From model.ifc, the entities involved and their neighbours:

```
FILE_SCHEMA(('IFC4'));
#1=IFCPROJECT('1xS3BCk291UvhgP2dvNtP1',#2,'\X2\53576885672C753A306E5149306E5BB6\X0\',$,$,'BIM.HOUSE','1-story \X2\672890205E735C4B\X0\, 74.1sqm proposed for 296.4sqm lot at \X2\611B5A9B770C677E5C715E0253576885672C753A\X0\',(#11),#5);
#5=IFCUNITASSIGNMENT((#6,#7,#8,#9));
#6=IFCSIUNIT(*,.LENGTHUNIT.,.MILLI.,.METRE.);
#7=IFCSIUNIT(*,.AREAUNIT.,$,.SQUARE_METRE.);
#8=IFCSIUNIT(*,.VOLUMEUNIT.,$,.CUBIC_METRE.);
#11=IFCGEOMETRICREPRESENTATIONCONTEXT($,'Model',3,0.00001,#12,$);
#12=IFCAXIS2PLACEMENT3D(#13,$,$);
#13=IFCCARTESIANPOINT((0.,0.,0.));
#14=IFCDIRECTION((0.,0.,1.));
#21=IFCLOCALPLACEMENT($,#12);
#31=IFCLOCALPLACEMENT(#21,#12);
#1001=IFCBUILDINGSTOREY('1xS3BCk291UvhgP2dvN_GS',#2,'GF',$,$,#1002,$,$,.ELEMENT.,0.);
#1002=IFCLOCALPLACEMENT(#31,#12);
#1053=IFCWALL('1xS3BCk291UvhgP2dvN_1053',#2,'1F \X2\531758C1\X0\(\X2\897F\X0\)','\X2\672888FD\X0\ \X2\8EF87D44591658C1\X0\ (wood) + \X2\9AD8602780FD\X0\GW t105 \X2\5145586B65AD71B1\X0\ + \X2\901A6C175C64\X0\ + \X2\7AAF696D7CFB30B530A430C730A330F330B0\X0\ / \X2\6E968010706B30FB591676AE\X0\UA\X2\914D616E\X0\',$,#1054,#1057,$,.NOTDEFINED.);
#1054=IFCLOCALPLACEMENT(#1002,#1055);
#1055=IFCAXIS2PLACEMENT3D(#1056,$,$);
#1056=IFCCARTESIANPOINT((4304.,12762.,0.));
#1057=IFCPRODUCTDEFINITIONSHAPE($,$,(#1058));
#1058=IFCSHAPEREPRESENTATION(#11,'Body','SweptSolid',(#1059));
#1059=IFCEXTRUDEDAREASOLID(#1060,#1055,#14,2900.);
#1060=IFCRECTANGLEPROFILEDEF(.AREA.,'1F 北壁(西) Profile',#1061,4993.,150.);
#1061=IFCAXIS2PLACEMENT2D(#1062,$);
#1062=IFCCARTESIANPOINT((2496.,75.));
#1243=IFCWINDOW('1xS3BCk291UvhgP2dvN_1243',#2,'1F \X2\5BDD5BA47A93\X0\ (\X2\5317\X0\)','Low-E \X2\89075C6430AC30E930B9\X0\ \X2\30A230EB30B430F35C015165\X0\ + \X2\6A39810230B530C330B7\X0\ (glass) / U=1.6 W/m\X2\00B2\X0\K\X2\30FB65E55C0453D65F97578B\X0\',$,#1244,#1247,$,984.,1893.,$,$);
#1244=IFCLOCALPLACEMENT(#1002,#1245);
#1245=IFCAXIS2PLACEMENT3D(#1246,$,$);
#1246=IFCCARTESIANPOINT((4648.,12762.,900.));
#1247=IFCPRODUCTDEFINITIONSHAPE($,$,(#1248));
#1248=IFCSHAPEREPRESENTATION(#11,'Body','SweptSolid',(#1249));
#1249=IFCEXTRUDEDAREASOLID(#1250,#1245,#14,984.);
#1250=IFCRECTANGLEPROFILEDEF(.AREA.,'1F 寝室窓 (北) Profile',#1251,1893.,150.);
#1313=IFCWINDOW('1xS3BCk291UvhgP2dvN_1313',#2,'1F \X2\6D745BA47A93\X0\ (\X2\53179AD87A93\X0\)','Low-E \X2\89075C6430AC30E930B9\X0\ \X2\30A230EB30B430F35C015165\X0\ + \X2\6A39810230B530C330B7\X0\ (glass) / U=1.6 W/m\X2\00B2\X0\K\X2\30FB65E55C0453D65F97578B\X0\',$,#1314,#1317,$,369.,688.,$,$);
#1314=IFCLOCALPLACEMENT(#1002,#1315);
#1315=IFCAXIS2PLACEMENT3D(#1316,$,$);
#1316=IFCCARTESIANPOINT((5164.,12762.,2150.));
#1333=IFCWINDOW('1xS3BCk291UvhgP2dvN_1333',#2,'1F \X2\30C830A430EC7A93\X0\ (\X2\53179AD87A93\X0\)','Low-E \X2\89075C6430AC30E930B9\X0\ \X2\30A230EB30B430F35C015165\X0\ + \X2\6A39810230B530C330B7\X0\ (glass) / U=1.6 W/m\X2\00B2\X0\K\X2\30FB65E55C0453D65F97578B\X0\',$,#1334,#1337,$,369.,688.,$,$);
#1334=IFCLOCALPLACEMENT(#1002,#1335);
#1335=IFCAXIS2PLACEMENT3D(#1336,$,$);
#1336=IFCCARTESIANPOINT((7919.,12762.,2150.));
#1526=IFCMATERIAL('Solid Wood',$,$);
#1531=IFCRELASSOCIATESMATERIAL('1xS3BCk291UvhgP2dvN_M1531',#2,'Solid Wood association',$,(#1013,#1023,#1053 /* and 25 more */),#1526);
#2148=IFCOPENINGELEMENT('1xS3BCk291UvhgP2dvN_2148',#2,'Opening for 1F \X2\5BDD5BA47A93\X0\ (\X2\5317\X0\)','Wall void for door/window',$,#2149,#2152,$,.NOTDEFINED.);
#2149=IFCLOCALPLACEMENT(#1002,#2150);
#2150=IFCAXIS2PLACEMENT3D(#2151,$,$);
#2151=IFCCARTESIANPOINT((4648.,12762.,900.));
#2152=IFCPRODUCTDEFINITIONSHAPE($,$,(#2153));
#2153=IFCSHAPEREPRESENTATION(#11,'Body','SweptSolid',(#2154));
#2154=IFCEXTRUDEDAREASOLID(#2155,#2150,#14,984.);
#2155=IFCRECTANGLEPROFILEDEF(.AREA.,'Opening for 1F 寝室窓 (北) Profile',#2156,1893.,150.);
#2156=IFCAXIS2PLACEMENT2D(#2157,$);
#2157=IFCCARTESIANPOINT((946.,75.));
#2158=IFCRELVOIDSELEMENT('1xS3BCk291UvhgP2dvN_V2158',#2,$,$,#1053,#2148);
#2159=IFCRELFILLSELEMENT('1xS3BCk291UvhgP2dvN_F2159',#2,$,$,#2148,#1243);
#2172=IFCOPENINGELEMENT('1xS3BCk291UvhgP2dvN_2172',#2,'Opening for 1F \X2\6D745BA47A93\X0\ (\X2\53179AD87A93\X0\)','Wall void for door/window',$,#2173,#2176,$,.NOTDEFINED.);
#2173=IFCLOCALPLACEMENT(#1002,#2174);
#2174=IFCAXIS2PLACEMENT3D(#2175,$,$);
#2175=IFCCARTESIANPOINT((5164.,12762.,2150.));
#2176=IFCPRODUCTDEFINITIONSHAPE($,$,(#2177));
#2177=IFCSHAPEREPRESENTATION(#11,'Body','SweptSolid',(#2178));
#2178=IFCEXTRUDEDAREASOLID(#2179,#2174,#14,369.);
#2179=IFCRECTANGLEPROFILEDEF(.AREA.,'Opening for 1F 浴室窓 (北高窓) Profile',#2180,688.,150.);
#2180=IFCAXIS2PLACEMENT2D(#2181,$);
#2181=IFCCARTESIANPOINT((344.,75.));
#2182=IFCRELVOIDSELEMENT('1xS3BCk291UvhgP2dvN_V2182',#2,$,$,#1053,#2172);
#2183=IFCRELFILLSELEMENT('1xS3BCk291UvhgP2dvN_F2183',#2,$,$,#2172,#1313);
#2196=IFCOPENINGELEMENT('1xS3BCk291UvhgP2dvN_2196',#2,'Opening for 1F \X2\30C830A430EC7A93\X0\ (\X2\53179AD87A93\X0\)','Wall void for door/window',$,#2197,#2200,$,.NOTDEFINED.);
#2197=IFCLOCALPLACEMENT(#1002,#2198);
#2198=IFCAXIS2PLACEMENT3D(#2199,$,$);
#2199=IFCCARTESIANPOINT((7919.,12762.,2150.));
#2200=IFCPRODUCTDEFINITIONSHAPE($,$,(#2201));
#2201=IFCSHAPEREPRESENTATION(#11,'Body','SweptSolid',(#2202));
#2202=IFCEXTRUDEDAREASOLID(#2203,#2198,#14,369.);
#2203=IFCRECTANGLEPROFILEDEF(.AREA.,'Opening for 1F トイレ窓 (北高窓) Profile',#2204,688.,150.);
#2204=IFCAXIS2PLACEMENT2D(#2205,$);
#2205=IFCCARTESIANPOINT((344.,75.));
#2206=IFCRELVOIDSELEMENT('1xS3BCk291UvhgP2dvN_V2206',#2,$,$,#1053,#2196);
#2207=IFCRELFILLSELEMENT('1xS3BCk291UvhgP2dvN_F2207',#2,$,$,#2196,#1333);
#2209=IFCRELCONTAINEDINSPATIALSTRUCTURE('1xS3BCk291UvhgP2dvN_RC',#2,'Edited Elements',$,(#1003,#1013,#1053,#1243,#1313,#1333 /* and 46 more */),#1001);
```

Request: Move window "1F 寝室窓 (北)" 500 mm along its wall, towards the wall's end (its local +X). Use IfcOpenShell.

```python
import ifcopenshell
import ifcopenshell.api.geometry
import ifcopenshell.util.placement
import ifcopenshell.util.unit

model = ifcopenshell.open("model.ifc")
unit_scale = ifcopenshell.util.unit.calculate_unit_scale(model)

window = model.by_guid("1xS3BCk291UvhgP2dvN_1243")
opening = window.FillsVoids[0].RelatingOpeningElement
wall = opening.VoidsElements[0].RelatingBuildingElement

wall_matrix = ifcopenshell.util.placement.get_local_placement(wall.ObjectPlacement)
shift = wall_matrix[:3, 0] * 0.5 / unit_scale
before = ifcopenshell.util.placement.get_local_placement(window.ObjectPlacement)[:3, 3].copy()

# The window is not placed relative to its opening, so move both.
for product in (opening, window):
    matrix = ifcopenshell.util.placement.get_local_placement(product.ObjectPlacement)
    matrix[:3, 3] += shift
    ifcopenshell.api.geometry.edit_object_placement(model, product=product, matrix=matrix, is_si=False)

after = ifcopenshell.util.placement.get_local_placement(window.ObjectPlacement)[:3, 3]
print("window moved by", (after - before).round(3) + 0.0)

model.write("model_rev.ifc")
```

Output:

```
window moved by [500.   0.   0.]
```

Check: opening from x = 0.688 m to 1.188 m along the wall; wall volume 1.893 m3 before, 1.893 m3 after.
